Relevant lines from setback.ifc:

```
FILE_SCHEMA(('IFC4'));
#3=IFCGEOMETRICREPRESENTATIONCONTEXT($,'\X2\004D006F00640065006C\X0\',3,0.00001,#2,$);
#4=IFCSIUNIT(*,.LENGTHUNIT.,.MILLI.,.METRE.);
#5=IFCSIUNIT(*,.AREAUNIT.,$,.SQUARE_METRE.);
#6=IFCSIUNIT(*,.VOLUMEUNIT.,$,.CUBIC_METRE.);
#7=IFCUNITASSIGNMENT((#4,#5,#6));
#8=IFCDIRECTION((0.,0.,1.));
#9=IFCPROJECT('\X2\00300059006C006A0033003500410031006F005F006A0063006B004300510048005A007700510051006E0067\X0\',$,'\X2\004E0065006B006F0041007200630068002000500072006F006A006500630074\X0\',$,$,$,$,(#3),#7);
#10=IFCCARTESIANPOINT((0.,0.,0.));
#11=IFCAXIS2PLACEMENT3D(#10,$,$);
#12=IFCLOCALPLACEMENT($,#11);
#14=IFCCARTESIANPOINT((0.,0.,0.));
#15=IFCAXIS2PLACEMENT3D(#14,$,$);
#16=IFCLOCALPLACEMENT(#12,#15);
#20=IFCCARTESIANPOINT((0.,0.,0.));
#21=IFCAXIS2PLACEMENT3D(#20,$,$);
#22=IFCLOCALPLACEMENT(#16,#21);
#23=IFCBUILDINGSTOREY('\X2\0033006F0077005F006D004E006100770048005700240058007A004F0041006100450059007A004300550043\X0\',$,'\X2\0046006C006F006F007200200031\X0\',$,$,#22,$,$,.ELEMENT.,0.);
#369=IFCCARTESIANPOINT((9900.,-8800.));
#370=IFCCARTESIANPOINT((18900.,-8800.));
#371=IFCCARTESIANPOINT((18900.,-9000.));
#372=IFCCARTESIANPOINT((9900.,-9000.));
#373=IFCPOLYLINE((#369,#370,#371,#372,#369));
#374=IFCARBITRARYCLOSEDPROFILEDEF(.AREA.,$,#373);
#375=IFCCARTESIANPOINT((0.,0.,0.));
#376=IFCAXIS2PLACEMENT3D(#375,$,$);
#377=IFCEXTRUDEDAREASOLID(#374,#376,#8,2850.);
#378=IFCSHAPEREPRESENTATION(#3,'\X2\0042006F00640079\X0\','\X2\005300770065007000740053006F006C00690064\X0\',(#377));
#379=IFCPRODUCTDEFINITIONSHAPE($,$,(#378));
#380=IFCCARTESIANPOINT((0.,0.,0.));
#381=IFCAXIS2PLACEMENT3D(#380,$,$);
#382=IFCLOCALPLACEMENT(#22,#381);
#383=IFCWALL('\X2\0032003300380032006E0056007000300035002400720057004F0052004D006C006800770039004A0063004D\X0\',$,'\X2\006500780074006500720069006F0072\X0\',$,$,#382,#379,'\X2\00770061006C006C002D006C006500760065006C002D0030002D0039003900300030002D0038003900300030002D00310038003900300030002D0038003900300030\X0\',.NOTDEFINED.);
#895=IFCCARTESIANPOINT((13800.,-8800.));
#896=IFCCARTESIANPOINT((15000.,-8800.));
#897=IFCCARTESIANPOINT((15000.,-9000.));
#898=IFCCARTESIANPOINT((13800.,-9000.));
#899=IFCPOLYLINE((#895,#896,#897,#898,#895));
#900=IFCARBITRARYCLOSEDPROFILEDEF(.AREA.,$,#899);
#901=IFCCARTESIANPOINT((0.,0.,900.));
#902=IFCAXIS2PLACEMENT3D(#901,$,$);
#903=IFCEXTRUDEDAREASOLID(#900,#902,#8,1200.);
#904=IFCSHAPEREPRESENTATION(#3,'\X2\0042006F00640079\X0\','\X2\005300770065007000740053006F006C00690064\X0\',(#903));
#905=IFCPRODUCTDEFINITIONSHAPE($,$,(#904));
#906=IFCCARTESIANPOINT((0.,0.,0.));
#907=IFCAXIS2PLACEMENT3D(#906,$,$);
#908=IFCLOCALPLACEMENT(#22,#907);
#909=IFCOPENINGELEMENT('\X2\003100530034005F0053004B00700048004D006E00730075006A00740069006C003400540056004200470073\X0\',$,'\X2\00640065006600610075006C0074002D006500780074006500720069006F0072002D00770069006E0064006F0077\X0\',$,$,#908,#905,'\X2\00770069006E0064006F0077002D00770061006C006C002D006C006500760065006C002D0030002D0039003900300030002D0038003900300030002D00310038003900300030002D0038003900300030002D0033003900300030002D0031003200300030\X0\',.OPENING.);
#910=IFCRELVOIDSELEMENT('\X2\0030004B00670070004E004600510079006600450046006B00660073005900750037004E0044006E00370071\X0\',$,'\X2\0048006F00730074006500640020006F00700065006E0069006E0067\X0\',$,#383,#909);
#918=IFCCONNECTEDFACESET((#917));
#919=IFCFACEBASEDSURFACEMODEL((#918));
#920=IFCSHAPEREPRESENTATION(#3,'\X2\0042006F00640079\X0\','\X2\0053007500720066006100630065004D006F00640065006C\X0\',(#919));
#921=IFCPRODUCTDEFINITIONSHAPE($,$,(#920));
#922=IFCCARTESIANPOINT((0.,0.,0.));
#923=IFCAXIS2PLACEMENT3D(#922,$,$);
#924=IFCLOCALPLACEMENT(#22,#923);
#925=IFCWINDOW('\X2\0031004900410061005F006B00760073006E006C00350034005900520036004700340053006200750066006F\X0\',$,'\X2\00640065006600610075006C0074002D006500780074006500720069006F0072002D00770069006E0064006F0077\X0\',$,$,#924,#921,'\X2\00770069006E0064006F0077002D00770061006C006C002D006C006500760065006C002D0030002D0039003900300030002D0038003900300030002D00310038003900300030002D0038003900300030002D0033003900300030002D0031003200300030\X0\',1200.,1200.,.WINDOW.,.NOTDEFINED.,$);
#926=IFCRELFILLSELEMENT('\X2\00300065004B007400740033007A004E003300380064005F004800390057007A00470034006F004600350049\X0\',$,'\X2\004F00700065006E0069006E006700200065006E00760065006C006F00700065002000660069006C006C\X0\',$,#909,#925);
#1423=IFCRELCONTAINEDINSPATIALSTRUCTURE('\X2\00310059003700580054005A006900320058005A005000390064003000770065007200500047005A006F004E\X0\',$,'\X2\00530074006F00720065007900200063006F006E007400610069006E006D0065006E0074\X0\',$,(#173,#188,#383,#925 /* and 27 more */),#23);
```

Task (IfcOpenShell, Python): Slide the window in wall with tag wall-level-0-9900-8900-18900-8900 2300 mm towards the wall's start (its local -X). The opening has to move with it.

```python
import ifcopenshell
import ifcopenshell.api.geometry
import ifcopenshell.util.placement
import ifcopenshell.util.unit

model = ifcopenshell.open("setback.ifc")
unit_scale = ifcopenshell.util.unit.calculate_unit_scale(model)

window = model.by_guid("1IAa_kvsnl54YR6G4Sbufo")
opening = window.FillsVoids[0].RelatingOpeningElement
wall = opening.VoidsElements[0].RelatingBuildingElement

wall_matrix = ifcopenshell.util.placement.get_local_placement(wall.ObjectPlacement)
shift = wall_matrix[:3, 0] * -2.3 / unit_scale
before = ifcopenshell.util.placement.get_local_placement(window.ObjectPlacement)[:3, 3].copy()

# The window is not placed relative to its opening, so move both.
for product in (opening, window):
    matrix = ifcopenshell.util.placement.get_local_placement(product.ObjectPlacement)
    matrix[:3, 3] += shift
    ifcopenshell.api.geometry.edit_object_placement(model, product=product, matrix=matrix, is_si=False)

after = ifcopenshell.util.placement.get_local_placement(window.ObjectPlacement)[:3, 3]
print("window moved by", (after - before).round(3) + 0.0)

model.write("setback_rev.ifc")
```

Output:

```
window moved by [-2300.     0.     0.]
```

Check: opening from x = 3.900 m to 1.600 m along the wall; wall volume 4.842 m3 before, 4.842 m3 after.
